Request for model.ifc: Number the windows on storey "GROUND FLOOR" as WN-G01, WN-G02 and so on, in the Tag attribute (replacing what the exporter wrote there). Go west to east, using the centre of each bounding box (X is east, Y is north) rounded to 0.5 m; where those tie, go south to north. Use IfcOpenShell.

First a look at what the model holds.

```python
import ifcopenshell
import ifcopenshell.util.element
import ifcopenshell.util.placement

model = ifcopenshell.open("model.ifc")
print(model.schema)
storey = next(s for s in model.by_type("IfcBuildingStorey") if s.Name == "GROUND FLOOR")
windows = [e for e in ifcopenshell.util.element.get_decomposition(storey) if e.is_a("IfcWindow")]
for e in sorted(windows, key=lambda e: e.id()):
    origin = ifcopenshell.util.placement.get_local_placement(e.ObjectPlacement)[:3, 3]
    print(e.id(), e.Tag, e.Name, origin.round(2) + 0.0, sep=" | ")
```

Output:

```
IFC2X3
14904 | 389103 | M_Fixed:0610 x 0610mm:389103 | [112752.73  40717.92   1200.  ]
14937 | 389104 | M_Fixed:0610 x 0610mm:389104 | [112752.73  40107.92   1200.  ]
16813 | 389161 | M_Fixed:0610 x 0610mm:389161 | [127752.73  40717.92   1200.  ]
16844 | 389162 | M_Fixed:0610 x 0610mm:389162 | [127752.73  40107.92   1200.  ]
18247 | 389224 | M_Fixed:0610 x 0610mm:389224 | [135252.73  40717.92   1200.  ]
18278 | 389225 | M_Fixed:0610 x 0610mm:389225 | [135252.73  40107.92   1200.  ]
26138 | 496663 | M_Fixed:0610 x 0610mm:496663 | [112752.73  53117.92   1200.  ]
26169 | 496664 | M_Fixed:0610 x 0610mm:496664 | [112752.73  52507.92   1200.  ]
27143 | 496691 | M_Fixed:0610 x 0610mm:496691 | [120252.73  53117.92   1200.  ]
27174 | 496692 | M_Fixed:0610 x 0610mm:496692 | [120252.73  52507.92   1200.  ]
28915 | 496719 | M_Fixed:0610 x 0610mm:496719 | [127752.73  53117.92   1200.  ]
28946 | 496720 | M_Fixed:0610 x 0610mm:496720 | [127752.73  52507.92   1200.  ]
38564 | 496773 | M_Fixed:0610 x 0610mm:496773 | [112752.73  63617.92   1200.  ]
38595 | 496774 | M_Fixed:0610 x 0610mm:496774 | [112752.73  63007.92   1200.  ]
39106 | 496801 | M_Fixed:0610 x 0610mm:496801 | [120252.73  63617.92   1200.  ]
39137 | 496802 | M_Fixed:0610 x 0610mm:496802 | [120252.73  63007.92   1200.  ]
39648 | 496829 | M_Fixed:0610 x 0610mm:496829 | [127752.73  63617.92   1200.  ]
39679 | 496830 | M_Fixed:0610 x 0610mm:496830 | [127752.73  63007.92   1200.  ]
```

```python
import ifcopenshell
import ifcopenshell.geom
import ifcopenshell.util.element
import ifcopenshell.util.shape

model = ifcopenshell.open("model.ifc")
settings = ifcopenshell.geom.settings()
settings.set("use-world-coords", True)


def centre(element):
    shape = ifcopenshell.geom.create_shape(settings, element)
    return ifcopenshell.util.shape.get_bbox_centroid(shape.geometry)


storey = next(s for s in model.by_type("IfcBuildingStorey") if s.Name == "GROUND FLOOR")
windows = [e for e in ifcopenshell.util.element.get_decomposition(storey) if e.is_a("IfcWindow")]

# Insertion points can sit at a corner or the storey origin, so sort by the geometry (in metres).
centres = {e: centre(e) for e in windows}
windows.sort(key=lambda e: (round(centres[e][0] / 0.5), centres[e][1]))

for i, e in enumerate(windows, start=1):
    number = f"WN-G{i:02d}"
    e.Tag = number
    print(e.id(), number)

model.write("model-out.ifc")
```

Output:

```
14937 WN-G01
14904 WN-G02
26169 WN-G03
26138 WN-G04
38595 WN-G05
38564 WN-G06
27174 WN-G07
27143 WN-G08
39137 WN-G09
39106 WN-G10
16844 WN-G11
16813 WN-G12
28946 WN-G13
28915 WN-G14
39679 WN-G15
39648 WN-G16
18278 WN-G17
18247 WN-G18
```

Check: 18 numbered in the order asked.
